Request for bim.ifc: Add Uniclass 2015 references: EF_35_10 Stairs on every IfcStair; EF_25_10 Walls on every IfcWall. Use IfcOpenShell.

First a look at what the model holds.

```python
import ifcopenshell

model = ifcopenshell.open("bim.ifc")
print(model.schema)
print("classifications:", [c.Name for c in model.by_type("IfcClassification")])
for ifc_class in ("IfcDoor", "IfcRoof", "IfcStair", "IfcWall", "IfcWindow"):
    print(ifc_class, len(model.by_type(ifc_class)))
```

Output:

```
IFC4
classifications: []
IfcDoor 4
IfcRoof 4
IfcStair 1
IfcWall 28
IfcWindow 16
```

```python
import ifcopenshell
import ifcopenshell.api.classification

model = ifcopenshell.open("bim.ifc")

system = ifcopenshell.api.classification.add_classification(model, classification="Uniclass 2015")

codes = {
    "IfcStair": ("EF_35_10", "Stairs"),
    "IfcWall": ("EF_25_10", "Walls"),
}
for ifc_class, (code, name) in codes.items():
    products = model.by_type(ifc_class)
    ifcopenshell.api.classification.add_reference(
        model, products=products, classification=system, identification=code, name=name
    )
    print(code, len(products))

model.write("bim-out.ifc")
```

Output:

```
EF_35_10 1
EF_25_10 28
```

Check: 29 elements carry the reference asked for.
